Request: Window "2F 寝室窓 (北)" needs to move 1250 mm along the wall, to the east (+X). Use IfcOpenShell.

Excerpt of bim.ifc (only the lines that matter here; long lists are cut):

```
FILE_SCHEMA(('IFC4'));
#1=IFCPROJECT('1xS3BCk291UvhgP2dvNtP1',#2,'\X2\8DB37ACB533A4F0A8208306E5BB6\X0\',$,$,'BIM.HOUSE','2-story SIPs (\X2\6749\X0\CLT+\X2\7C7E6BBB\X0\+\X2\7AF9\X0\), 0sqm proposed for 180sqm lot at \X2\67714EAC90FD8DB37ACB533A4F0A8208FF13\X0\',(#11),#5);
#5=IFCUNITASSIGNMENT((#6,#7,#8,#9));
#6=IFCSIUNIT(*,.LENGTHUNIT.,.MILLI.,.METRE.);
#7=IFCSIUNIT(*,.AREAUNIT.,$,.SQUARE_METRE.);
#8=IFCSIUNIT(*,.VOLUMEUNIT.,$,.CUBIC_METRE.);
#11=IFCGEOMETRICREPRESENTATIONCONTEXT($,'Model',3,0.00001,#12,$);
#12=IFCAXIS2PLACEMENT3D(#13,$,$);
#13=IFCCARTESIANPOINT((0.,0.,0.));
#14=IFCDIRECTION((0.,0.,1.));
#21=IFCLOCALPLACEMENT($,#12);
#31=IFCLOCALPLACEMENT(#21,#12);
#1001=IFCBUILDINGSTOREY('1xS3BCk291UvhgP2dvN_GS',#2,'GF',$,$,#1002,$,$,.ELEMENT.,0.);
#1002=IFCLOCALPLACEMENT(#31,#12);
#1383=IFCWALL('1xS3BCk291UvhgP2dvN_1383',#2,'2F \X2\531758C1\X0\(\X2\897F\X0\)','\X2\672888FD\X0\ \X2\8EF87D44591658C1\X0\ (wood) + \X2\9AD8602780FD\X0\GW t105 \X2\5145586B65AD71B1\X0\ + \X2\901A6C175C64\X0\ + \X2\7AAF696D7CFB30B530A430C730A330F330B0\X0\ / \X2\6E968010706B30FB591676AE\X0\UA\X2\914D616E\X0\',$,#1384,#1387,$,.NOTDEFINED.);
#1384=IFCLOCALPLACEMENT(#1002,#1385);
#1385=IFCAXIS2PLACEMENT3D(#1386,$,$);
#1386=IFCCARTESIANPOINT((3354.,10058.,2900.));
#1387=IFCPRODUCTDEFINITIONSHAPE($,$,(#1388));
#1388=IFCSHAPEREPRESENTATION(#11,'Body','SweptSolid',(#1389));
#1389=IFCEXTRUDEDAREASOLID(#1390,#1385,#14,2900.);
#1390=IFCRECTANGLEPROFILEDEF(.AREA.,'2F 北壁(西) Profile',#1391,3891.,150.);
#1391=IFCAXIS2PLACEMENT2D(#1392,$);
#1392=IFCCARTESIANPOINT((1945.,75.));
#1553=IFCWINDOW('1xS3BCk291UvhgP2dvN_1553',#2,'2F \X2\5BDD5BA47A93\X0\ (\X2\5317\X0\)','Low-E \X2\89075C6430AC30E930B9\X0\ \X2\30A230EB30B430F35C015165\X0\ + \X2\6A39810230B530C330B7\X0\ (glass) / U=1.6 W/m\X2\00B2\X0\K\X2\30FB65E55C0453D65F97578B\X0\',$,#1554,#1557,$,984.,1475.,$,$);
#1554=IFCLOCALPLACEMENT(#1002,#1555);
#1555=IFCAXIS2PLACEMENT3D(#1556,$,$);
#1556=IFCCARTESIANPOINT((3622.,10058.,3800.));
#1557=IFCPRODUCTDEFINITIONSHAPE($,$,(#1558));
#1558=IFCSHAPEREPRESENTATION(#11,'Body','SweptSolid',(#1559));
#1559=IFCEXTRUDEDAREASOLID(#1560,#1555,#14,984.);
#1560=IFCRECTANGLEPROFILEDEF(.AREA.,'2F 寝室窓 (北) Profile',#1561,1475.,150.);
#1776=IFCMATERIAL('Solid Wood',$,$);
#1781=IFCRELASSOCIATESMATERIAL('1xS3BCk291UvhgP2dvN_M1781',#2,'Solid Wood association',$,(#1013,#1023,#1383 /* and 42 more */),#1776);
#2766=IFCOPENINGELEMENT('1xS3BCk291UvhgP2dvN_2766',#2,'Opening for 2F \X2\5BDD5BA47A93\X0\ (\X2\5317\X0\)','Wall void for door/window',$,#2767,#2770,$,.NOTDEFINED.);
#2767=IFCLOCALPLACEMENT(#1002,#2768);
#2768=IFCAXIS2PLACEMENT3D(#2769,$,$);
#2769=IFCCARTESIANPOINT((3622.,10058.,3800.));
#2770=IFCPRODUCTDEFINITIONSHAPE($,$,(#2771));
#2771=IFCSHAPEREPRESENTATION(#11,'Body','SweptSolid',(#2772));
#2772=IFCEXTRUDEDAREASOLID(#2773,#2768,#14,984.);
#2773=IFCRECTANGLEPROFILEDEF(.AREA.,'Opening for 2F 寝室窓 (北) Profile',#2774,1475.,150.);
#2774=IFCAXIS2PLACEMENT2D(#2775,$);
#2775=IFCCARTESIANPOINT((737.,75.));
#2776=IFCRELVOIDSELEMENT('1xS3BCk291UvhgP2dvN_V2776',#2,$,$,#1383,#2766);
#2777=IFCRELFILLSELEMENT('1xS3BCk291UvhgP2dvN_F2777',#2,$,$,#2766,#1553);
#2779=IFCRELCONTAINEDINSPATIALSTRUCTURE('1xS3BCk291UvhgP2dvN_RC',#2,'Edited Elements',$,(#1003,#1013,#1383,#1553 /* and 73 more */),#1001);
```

```python
import ifcopenshell
import ifcopenshell.api.geometry
import ifcopenshell.util.placement
import ifcopenshell.util.unit

model = ifcopenshell.open("bim.ifc")
unit_scale = ifcopenshell.util.unit.calculate_unit_scale(model)

window = model.by_id(1553)
opening = window.FillsVoids[0].RelatingOpeningElement
wall = opening.VoidsElements[0].RelatingBuildingElement

wall_matrix = ifcopenshell.util.placement.get_local_placement(wall.ObjectPlacement)
shift = wall_matrix[:3, 0] * 1.25 / unit_scale
before = ifcopenshell.util.placement.get_local_placement(window.ObjectPlacement)[:3, 3].copy()

# The window is not placed relative to its opening, so move both.
for product in (opening, window):
    matrix = ifcopenshell.util.placement.get_local_placement(product.ObjectPlacement)
    matrix[:3, 3] += shift
    ifcopenshell.api.geometry.edit_object_placement(model, product=product, matrix=matrix, is_si=False)

after = ifcopenshell.util.placement.get_local_placement(window.ObjectPlacement)[:3, 3]
print("window moved by", (after - before).round(3) + 0.0)

model.write("bim-out.ifc")
```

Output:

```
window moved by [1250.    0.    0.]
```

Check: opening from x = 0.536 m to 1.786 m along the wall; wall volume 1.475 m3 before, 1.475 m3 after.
